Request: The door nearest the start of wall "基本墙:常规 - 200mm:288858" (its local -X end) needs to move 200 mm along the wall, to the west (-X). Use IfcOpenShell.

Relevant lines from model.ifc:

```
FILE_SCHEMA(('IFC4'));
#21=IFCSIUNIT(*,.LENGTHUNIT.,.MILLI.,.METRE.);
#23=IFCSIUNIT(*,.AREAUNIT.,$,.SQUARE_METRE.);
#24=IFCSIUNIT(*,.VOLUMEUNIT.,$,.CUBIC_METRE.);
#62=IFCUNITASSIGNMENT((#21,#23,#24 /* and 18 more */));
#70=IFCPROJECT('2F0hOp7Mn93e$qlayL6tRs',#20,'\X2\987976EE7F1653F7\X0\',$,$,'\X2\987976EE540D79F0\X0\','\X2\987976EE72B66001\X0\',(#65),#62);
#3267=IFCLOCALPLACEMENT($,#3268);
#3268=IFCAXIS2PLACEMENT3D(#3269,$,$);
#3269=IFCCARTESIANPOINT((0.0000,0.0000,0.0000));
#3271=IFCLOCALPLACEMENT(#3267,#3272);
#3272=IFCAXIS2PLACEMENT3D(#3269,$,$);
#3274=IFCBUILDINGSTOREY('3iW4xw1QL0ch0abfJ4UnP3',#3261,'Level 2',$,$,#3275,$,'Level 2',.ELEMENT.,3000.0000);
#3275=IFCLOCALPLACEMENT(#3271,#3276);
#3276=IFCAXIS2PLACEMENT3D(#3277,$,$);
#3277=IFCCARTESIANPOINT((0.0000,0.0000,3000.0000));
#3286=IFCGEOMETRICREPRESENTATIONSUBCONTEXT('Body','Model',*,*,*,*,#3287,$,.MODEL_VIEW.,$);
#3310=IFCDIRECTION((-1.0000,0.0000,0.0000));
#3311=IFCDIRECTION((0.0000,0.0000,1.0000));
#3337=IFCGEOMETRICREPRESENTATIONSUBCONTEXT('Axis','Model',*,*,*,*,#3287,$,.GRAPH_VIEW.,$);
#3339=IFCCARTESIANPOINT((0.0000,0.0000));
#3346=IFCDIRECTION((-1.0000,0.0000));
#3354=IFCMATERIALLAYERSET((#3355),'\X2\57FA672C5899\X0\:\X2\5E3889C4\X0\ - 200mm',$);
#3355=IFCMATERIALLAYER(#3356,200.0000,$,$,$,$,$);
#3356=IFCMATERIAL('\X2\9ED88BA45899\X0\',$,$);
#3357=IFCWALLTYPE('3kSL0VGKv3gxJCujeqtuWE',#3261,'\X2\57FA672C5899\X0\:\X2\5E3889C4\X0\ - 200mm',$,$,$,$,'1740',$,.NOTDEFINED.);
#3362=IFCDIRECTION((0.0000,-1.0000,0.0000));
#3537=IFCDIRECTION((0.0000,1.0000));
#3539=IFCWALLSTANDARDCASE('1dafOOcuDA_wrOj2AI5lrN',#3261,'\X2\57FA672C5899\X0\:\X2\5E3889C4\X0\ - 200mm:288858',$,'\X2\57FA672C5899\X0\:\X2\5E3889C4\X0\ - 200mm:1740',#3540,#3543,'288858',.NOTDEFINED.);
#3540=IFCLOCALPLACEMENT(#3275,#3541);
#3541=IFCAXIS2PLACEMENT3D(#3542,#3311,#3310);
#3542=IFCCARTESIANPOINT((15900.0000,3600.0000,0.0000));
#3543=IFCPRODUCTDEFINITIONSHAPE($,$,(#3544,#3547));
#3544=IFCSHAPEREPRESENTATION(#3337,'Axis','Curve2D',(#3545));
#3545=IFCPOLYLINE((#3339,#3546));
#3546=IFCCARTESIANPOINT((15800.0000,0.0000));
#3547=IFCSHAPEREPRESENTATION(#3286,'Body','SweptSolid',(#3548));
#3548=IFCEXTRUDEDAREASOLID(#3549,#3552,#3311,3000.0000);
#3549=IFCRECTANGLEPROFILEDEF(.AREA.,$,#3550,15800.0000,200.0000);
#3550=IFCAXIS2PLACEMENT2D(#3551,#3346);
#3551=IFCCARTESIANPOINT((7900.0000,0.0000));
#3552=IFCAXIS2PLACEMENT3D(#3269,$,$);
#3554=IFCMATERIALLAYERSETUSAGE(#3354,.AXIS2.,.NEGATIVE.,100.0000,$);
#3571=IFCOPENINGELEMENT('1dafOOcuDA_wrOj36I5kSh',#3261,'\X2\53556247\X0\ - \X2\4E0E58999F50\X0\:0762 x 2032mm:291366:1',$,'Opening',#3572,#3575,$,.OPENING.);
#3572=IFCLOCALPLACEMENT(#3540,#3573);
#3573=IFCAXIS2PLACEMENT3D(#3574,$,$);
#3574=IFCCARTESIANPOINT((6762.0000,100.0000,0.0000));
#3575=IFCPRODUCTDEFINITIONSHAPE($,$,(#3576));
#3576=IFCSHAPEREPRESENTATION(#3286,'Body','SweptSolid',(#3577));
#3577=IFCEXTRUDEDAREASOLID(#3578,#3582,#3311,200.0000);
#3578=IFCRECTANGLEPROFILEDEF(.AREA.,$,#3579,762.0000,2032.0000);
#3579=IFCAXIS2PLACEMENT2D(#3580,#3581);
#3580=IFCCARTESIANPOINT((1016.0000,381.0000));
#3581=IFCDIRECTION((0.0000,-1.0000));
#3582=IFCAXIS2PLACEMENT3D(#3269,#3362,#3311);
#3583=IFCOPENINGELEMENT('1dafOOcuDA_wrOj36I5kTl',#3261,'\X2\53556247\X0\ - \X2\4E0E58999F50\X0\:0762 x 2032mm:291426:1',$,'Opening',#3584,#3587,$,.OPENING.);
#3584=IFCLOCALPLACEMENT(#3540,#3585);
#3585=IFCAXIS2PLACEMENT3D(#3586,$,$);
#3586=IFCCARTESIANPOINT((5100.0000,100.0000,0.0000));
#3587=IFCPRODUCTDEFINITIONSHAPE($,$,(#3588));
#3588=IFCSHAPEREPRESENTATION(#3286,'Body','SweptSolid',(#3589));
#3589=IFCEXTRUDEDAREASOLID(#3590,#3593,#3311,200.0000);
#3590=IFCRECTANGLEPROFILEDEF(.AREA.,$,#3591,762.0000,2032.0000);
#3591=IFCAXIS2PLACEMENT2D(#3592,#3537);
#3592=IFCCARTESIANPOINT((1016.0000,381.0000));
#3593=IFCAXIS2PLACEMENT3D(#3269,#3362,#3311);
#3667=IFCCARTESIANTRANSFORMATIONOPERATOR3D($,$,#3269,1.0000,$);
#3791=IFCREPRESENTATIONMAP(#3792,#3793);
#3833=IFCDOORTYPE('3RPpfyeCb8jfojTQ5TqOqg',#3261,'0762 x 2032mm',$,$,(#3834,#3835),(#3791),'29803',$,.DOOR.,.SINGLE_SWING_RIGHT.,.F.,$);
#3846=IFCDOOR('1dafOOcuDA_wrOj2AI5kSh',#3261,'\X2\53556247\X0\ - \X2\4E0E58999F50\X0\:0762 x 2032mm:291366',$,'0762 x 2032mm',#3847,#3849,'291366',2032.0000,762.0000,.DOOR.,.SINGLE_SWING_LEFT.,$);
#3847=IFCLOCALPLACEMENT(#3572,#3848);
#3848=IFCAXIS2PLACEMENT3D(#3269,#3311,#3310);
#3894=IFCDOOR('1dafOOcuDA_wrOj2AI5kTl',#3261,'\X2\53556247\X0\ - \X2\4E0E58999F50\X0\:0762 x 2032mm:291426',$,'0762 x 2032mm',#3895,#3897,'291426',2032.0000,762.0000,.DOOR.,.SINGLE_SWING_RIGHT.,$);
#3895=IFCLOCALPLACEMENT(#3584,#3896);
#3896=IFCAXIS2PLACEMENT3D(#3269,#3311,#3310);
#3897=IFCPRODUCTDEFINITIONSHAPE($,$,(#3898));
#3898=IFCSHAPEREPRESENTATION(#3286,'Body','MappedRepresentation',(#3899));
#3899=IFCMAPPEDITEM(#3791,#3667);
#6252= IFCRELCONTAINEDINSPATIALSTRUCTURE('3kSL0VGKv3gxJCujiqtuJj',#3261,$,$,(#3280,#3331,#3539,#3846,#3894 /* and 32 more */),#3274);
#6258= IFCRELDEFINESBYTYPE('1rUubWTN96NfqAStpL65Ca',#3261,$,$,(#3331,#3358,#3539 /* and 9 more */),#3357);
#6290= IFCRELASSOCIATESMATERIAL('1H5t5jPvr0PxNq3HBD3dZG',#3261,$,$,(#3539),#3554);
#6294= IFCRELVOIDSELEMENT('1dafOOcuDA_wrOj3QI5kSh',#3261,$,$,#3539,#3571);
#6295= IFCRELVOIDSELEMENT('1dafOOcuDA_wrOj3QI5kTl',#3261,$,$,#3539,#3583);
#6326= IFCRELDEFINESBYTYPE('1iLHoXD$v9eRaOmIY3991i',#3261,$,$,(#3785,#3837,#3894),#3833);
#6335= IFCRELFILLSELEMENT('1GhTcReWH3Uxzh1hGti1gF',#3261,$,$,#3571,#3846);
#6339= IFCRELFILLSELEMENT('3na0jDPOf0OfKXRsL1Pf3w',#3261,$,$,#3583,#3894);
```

```python
import ifcopenshell
import ifcopenshell.api.geometry
import ifcopenshell.util.placement

model = ifcopenshell.open("model.ifc")

door = model.by_guid("1dafOOcuDA_wrOj2AI5kTl")
opening = door.FillsVoids[0].RelatingOpeningElement
wall = opening.VoidsElements[0].RelatingBuildingElement

wall_matrix = ifcopenshell.util.placement.get_local_placement(wall.ObjectPlacement)
shift = wall_matrix[:3, 0] * 200.0
before = ifcopenshell.util.placement.get_local_placement(door.ObjectPlacement)[:3, 3].copy()

# The door is placed relative to its opening, so it follows when the opening moves.
matrix = ifcopenshell.util.placement.get_local_placement(opening.ObjectPlacement)
matrix[:3, 3] += shift
ifcopenshell.api.geometry.edit_object_placement(
    model, product=opening, matrix=matrix, is_si=False, should_transform_children=True
)

after = ifcopenshell.util.placement.get_local_placement(door.ObjectPlacement)[:3, 3]
print("door moved by", (after - before).round(3) + 0.0)

model.write("model_updated.ifc")
```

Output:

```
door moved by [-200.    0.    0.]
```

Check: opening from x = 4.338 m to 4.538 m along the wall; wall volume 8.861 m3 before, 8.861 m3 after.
